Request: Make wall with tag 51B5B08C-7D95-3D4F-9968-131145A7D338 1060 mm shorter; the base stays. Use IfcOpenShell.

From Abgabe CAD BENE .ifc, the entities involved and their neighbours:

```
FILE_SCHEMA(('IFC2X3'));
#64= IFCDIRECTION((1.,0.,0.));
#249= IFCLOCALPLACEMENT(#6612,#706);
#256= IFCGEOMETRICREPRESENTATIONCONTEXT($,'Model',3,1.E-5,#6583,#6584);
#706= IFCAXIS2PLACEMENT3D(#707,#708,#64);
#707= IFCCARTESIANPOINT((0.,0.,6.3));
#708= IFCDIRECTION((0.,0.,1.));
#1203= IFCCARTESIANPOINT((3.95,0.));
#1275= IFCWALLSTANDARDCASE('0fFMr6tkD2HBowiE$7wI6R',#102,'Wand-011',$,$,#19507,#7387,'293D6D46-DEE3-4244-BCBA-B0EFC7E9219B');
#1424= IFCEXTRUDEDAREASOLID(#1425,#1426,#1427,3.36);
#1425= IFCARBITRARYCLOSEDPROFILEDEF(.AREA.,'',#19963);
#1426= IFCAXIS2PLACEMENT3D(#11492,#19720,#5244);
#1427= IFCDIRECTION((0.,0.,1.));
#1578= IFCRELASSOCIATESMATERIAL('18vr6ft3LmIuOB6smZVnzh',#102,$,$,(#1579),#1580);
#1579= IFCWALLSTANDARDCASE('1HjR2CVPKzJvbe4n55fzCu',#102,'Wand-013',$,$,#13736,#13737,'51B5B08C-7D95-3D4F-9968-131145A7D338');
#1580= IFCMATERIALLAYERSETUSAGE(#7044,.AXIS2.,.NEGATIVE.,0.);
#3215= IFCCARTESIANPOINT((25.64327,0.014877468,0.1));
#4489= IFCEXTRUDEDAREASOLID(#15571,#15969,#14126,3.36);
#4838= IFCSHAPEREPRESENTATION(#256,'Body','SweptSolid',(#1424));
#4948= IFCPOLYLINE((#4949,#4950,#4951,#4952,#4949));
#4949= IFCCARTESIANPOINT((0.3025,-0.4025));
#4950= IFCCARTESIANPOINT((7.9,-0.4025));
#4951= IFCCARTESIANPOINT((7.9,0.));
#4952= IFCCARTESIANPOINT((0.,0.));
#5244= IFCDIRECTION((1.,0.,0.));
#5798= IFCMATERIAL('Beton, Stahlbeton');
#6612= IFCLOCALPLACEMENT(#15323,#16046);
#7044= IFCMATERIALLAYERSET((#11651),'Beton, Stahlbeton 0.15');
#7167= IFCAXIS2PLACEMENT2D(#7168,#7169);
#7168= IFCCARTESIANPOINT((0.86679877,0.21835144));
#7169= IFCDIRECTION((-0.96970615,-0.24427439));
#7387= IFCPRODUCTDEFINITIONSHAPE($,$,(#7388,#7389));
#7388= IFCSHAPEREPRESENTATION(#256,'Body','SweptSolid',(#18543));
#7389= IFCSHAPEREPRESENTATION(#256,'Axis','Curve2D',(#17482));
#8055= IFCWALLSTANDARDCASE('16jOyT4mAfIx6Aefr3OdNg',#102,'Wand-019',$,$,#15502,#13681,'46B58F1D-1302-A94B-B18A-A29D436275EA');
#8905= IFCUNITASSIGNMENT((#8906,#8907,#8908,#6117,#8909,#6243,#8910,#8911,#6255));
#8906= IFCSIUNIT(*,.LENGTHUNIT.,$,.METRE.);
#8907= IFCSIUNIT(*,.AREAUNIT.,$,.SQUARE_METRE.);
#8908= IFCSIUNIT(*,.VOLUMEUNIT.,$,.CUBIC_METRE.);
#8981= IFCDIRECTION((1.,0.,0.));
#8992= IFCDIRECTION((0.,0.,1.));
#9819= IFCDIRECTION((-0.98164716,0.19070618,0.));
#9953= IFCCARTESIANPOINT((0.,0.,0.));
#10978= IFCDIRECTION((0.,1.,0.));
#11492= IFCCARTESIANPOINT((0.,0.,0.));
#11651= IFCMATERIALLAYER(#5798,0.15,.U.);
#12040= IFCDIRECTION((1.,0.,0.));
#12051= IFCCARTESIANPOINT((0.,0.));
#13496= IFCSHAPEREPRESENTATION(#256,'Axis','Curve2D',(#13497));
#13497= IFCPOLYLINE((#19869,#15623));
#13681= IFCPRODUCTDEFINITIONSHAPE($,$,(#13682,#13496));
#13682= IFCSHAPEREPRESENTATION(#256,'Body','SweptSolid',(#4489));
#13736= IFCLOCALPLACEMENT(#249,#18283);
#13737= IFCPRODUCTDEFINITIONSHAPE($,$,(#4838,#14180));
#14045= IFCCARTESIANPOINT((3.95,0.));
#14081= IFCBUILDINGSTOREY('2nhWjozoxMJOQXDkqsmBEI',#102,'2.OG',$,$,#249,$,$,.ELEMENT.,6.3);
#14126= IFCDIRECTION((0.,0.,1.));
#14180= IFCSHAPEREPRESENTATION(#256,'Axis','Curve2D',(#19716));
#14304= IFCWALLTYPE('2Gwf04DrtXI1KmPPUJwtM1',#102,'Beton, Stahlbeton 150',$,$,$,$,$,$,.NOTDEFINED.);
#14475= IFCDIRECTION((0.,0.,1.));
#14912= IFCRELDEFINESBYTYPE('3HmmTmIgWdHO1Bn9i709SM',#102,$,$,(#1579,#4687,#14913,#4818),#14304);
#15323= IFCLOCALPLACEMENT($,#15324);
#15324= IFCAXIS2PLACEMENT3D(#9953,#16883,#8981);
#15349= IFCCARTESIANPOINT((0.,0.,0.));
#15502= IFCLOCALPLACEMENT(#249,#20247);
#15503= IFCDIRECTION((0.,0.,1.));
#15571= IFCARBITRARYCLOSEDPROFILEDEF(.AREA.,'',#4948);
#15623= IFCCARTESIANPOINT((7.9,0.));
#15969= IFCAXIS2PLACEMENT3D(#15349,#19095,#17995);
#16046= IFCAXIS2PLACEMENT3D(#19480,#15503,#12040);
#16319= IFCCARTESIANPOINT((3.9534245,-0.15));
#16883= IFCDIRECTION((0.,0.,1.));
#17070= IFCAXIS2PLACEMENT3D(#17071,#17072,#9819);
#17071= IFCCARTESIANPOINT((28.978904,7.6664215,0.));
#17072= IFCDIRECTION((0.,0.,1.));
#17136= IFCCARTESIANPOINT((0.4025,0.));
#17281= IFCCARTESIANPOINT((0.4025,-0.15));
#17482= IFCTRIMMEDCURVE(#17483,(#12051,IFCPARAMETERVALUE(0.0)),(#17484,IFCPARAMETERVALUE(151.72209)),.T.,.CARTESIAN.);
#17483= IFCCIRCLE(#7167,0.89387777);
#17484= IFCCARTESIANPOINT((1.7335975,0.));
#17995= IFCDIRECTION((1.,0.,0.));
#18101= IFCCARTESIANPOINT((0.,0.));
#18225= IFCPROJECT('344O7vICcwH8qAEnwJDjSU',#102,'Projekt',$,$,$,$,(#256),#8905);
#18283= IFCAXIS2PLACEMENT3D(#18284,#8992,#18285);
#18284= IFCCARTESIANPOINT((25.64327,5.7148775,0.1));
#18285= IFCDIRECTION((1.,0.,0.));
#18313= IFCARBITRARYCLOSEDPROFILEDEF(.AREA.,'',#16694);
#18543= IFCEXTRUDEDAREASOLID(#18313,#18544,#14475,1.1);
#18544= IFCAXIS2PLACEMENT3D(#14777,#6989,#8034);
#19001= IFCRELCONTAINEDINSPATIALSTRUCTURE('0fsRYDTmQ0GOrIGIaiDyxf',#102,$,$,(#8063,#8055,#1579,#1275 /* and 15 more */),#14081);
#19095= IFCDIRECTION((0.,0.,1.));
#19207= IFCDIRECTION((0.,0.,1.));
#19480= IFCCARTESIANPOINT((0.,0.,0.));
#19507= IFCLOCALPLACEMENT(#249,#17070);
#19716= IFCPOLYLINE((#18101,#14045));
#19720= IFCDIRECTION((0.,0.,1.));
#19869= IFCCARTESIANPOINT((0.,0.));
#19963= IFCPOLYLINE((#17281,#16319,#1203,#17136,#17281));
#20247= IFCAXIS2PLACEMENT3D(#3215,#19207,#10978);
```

```python
import ifcopenshell
import ifcopenshell.geom
import ifcopenshell.util.shape

model = ifcopenshell.open("Abgabe CAD BENE .ifc")
settings = ifcopenshell.geom.settings()


def volume(element):
    """Net volume in cubic metres, openings subtracted."""
    shape = ifcopenshell.geom.create_shape(settings, element)
    return ifcopenshell.util.shape.get_volume(shape.geometry)


wall = model.by_guid("1HjR2CVPKzJvbe4n55fzCu")
before = volume(wall)

body = next(r for r in wall.Representation.Representations if r.RepresentationIdentifier == "Body")
solid = body.Items[0]
old_height = solid.Depth
solid.Depth -= 1.06
after = volume(wall)

print(f"height {old_height:g} -> {solid.Depth:g}, volume {before:.3f} -> {after:.3f} m3")

model.write("Abgabe CAD BENE _rev.ifc")
```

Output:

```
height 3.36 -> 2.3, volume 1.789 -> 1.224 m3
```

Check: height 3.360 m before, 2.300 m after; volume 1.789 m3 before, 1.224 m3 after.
